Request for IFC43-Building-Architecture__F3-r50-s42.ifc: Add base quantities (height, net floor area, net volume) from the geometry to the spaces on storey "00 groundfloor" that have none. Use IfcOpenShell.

First a look at what the model holds.

```python
import ifcopenshell
import ifcopenshell.util.element
import ifcopenshell.util.unit

model = ifcopenshell.open("IFC43-Building-Architecture__F3-r50-s42.ifc")
print(model.schema)
for unit_type in ("LENGTHUNIT", "AREAUNIT", "VOLUMEUNIT"):
    print(unit_type, ifcopenshell.util.unit.calculate_unit_scale(model, unit_type))
storey = next(s for s in model.by_type("IfcBuildingStorey") if s.Name == "00 groundfloor")
spaces = [e for e in ifcopenshell.util.element.get_decomposition(storey) if e.is_a("IfcSpace")]
for e in sorted(spaces, key=lambda e: e.id()):
    print(e.id(), e.is_a(), e.Name, list(ifcopenshell.util.element.get_psets(e, qtos_only=True)), sep=" | ")
```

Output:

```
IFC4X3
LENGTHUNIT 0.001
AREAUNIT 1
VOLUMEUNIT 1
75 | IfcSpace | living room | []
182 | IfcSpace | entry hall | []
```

```python
import ifcopenshell
import ifcopenshell.api.pset
import ifcopenshell.geom
import ifcopenshell.util.element
import ifcopenshell.util.shape
import ifcopenshell.util.unit

model = ifcopenshell.open("IFC43-Building-Architecture__F3-r50-s42.ifc")
unit_scale = ifcopenshell.util.unit.calculate_unit_scale(model)
area_scale = ifcopenshell.util.unit.calculate_unit_scale(model, "AREAUNIT")
volume_scale = ifcopenshell.util.unit.calculate_unit_scale(model, "VOLUMEUNIT")
settings = ifcopenshell.geom.settings()

storey = next(s for s in model.by_type("IfcBuildingStorey") if s.Name == "00 groundfloor")
spaces = [e for e in ifcopenshell.util.element.get_decomposition(storey) if e.is_a("IfcSpace")]

for e in sorted(spaces, key=lambda e: e.id()):
    if ifcopenshell.util.element.get_psets(e, qtos_only=True, should_inherit=False):
        continue
    # Geometry comes back in metres, in the element's own axes.
    shape = ifcopenshell.geom.create_shape(settings, e)
    values = {
        "Height": ifcopenshell.util.shape.get_z(shape.geometry) / unit_scale,
        "NetFloorArea": ifcopenshell.util.shape.get_footprint_area(shape.geometry) / area_scale,
        "NetVolume": ifcopenshell.util.shape.get_volume(shape.geometry) / volume_scale,
    }
    qto = ifcopenshell.api.pset.add_qto(model, product=e, name="Qto_SpaceBaseQuantities")
    ifcopenshell.api.pset.edit_qto(model, qto=qto, properties=values)
    print(e.id(), {k: round(v, 3) for k, v in values.items()})

model.write("IFC43-Building-Architecture__F3-r50-s42_edited.ifc")
```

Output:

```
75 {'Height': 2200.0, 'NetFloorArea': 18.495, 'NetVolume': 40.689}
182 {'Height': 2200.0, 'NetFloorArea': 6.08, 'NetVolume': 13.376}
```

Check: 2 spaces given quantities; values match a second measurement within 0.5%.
